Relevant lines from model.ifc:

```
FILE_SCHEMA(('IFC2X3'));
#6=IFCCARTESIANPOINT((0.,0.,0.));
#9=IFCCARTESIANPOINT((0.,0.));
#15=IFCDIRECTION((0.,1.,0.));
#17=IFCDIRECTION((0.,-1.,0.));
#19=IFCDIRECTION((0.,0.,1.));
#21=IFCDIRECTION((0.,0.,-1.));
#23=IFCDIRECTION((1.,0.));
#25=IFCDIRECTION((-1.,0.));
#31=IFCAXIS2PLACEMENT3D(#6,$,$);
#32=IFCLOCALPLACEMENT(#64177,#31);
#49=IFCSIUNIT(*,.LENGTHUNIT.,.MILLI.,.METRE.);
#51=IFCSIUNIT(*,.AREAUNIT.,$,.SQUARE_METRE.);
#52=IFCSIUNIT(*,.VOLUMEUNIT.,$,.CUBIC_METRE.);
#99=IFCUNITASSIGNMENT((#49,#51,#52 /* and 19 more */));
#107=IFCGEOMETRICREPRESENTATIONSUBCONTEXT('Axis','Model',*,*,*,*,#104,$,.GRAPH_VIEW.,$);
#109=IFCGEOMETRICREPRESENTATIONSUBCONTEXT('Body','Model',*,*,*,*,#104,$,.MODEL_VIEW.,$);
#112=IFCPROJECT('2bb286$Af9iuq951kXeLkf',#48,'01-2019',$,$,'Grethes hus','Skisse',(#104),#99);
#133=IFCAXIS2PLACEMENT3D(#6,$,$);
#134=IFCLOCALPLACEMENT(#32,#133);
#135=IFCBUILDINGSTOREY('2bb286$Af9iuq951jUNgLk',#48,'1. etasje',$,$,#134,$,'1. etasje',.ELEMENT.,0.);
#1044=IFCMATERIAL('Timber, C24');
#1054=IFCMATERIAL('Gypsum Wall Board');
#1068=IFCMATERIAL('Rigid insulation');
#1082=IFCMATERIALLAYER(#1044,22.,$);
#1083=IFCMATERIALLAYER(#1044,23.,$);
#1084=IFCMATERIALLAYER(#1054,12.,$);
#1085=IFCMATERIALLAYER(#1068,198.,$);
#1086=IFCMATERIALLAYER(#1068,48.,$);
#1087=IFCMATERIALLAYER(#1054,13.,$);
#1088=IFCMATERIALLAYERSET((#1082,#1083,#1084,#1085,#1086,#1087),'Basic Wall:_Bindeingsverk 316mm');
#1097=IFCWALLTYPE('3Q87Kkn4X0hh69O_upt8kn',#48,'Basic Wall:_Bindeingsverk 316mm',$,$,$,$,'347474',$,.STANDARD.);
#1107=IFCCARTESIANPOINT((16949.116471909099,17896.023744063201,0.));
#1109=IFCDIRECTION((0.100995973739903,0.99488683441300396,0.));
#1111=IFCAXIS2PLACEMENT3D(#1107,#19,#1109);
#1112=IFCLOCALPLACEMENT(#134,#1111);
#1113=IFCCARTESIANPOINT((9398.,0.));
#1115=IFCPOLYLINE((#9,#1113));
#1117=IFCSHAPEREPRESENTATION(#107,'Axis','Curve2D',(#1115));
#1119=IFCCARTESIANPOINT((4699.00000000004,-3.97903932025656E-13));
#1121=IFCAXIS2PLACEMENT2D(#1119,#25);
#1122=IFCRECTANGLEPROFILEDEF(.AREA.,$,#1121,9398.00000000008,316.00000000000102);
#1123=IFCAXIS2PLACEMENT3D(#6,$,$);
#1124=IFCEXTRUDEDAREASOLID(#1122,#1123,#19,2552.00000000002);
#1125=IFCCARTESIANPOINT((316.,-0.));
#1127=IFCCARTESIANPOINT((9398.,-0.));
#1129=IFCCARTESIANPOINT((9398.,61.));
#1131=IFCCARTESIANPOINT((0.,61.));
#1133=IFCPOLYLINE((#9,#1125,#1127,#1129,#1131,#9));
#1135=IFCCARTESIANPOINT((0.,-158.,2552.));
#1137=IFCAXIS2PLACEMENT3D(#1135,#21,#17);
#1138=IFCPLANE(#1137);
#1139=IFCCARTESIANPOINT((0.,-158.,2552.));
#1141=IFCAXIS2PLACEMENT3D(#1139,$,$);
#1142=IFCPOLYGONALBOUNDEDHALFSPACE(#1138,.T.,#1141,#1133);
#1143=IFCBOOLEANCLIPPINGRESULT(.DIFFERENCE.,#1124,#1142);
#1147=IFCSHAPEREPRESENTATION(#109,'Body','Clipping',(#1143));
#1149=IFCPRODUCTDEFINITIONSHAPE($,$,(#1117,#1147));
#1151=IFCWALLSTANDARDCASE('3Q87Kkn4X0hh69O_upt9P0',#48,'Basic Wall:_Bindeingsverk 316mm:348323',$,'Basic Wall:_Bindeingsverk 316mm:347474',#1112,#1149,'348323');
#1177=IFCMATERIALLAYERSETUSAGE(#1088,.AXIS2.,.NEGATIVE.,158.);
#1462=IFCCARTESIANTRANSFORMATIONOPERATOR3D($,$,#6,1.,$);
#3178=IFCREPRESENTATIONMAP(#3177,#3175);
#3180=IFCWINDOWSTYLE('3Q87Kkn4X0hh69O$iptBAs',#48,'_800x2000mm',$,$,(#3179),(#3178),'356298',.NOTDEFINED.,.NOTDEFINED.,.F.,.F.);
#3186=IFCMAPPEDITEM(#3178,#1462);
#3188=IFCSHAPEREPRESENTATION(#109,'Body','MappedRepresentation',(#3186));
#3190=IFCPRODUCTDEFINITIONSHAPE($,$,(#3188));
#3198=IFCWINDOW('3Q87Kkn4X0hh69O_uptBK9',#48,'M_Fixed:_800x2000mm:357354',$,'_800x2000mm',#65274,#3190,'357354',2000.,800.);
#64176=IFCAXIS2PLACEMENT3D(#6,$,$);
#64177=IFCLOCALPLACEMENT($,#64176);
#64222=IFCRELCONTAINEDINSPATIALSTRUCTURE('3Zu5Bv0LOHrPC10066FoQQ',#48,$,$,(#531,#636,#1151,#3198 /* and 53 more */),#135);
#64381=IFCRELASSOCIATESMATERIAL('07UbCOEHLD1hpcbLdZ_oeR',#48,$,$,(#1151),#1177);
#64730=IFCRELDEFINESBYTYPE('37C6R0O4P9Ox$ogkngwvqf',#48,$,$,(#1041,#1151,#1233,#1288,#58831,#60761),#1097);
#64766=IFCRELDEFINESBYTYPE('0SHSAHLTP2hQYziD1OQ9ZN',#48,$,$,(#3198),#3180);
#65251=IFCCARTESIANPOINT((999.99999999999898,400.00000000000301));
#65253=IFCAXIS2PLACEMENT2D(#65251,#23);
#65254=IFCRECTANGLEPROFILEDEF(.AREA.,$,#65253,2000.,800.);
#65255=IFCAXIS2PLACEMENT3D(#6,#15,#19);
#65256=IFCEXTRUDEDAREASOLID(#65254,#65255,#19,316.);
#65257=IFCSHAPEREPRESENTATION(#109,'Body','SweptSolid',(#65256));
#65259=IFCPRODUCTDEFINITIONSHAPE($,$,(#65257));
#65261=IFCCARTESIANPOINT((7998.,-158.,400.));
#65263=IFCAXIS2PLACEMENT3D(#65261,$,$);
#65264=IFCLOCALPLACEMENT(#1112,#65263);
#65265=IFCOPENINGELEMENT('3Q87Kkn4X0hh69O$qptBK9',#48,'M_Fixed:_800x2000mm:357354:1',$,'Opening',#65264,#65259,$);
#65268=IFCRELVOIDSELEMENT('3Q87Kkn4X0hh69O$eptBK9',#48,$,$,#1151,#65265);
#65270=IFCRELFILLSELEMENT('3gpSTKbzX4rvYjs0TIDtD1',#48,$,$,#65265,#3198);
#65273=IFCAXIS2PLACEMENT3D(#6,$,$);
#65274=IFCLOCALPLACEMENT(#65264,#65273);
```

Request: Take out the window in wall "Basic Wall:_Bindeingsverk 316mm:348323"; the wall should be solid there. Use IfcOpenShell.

```python
import ifcopenshell
import ifcopenshell.api.feature
import ifcopenshell.api.root
import ifcopenshell.geom
import ifcopenshell.util.shape

model = ifcopenshell.open("model.ifc")
settings = ifcopenshell.geom.settings()


def volume(element):
    """Net volume in cubic metres, openings subtracted."""
    shape = ifcopenshell.geom.create_shape(settings, element)
    return ifcopenshell.util.shape.get_volume(shape.geometry)


window = model.by_guid("3Q87Kkn4X0hh69O_uptBK9")
opening = window.FillsVoids[0].RelatingOpeningElement
wall = opening.VoidsElements[0].RelatingBuildingElement
before = volume(wall)

ifcopenshell.api.root.remove_product(model, product=window)
ifcopenshell.api.feature.remove_feature(model, feature=opening)

after = volume(wall)

print(f"wall volume {before:.3f} -> {after:.3f} m3")

model.write("model-out.ifc")
```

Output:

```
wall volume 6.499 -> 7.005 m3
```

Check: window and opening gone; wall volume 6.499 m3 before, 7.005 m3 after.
